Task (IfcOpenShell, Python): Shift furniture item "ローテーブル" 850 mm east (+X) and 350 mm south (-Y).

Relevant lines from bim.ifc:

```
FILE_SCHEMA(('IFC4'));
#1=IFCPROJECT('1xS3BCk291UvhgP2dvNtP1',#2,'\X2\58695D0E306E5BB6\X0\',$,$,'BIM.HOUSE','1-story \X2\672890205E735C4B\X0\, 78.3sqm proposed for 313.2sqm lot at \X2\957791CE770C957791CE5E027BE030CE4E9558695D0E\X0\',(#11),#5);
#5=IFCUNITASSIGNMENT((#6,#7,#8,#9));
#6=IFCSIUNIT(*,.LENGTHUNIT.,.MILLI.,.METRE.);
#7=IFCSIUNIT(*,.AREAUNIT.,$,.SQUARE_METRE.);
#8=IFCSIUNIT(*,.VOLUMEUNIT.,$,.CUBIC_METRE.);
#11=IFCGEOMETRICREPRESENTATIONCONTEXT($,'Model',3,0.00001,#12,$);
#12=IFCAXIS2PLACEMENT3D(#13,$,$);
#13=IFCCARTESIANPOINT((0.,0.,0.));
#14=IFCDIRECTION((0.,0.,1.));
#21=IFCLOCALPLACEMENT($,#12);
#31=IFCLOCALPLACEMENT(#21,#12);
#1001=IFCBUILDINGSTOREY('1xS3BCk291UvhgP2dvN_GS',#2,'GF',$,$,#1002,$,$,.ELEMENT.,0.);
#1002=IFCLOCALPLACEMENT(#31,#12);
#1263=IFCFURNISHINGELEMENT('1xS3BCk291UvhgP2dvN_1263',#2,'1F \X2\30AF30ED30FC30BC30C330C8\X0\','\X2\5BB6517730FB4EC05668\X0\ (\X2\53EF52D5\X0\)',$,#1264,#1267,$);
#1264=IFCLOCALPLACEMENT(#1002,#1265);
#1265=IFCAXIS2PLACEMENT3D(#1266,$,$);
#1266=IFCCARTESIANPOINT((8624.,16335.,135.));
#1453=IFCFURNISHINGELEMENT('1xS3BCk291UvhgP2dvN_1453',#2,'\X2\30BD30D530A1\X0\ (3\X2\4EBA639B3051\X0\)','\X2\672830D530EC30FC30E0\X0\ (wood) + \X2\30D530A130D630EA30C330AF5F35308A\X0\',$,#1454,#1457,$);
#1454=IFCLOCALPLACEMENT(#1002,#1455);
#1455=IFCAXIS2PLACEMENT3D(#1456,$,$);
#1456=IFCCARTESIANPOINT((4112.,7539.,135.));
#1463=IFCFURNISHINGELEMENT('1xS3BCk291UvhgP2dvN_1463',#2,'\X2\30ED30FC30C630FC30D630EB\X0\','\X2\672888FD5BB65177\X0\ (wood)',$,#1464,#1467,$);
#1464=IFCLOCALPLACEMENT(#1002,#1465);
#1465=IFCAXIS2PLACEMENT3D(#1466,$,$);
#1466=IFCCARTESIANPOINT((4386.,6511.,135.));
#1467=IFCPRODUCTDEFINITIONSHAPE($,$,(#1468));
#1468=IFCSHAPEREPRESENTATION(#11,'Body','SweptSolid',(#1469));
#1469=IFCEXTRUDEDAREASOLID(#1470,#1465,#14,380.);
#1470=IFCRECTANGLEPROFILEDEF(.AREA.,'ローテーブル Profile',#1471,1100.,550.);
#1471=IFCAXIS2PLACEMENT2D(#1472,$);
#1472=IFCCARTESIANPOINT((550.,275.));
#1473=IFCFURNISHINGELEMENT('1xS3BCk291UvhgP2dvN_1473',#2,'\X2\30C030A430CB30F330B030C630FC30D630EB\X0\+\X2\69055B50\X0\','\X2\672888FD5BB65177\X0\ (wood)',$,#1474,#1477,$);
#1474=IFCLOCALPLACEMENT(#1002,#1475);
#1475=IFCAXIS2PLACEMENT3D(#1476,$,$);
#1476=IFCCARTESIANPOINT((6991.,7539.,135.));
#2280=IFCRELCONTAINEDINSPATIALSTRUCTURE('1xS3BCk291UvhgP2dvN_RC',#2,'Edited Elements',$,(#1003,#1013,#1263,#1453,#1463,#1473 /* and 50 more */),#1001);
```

```python
import ifcopenshell
import ifcopenshell.api.geometry
import ifcopenshell.util.placement

model = ifcopenshell.open("bim.ifc")

item = model.by_guid("1xS3BCk291UvhgP2dvN_1463")
matrix = ifcopenshell.util.placement.get_local_placement(item.ObjectPlacement)
matrix[0, 3] += 850.0
matrix[1, 3] -= 350.0
ifcopenshell.api.geometry.edit_object_placement(model, product=item, matrix=matrix, is_si=False)

print(ifcopenshell.util.placement.get_local_placement(item.ObjectPlacement).round(3) + 0.0)

model.write("bim_v2.ifc")
```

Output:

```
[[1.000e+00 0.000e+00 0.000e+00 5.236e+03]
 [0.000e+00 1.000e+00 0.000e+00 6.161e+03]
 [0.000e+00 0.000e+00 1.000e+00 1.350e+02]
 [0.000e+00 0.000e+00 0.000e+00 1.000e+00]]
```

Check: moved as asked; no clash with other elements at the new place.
